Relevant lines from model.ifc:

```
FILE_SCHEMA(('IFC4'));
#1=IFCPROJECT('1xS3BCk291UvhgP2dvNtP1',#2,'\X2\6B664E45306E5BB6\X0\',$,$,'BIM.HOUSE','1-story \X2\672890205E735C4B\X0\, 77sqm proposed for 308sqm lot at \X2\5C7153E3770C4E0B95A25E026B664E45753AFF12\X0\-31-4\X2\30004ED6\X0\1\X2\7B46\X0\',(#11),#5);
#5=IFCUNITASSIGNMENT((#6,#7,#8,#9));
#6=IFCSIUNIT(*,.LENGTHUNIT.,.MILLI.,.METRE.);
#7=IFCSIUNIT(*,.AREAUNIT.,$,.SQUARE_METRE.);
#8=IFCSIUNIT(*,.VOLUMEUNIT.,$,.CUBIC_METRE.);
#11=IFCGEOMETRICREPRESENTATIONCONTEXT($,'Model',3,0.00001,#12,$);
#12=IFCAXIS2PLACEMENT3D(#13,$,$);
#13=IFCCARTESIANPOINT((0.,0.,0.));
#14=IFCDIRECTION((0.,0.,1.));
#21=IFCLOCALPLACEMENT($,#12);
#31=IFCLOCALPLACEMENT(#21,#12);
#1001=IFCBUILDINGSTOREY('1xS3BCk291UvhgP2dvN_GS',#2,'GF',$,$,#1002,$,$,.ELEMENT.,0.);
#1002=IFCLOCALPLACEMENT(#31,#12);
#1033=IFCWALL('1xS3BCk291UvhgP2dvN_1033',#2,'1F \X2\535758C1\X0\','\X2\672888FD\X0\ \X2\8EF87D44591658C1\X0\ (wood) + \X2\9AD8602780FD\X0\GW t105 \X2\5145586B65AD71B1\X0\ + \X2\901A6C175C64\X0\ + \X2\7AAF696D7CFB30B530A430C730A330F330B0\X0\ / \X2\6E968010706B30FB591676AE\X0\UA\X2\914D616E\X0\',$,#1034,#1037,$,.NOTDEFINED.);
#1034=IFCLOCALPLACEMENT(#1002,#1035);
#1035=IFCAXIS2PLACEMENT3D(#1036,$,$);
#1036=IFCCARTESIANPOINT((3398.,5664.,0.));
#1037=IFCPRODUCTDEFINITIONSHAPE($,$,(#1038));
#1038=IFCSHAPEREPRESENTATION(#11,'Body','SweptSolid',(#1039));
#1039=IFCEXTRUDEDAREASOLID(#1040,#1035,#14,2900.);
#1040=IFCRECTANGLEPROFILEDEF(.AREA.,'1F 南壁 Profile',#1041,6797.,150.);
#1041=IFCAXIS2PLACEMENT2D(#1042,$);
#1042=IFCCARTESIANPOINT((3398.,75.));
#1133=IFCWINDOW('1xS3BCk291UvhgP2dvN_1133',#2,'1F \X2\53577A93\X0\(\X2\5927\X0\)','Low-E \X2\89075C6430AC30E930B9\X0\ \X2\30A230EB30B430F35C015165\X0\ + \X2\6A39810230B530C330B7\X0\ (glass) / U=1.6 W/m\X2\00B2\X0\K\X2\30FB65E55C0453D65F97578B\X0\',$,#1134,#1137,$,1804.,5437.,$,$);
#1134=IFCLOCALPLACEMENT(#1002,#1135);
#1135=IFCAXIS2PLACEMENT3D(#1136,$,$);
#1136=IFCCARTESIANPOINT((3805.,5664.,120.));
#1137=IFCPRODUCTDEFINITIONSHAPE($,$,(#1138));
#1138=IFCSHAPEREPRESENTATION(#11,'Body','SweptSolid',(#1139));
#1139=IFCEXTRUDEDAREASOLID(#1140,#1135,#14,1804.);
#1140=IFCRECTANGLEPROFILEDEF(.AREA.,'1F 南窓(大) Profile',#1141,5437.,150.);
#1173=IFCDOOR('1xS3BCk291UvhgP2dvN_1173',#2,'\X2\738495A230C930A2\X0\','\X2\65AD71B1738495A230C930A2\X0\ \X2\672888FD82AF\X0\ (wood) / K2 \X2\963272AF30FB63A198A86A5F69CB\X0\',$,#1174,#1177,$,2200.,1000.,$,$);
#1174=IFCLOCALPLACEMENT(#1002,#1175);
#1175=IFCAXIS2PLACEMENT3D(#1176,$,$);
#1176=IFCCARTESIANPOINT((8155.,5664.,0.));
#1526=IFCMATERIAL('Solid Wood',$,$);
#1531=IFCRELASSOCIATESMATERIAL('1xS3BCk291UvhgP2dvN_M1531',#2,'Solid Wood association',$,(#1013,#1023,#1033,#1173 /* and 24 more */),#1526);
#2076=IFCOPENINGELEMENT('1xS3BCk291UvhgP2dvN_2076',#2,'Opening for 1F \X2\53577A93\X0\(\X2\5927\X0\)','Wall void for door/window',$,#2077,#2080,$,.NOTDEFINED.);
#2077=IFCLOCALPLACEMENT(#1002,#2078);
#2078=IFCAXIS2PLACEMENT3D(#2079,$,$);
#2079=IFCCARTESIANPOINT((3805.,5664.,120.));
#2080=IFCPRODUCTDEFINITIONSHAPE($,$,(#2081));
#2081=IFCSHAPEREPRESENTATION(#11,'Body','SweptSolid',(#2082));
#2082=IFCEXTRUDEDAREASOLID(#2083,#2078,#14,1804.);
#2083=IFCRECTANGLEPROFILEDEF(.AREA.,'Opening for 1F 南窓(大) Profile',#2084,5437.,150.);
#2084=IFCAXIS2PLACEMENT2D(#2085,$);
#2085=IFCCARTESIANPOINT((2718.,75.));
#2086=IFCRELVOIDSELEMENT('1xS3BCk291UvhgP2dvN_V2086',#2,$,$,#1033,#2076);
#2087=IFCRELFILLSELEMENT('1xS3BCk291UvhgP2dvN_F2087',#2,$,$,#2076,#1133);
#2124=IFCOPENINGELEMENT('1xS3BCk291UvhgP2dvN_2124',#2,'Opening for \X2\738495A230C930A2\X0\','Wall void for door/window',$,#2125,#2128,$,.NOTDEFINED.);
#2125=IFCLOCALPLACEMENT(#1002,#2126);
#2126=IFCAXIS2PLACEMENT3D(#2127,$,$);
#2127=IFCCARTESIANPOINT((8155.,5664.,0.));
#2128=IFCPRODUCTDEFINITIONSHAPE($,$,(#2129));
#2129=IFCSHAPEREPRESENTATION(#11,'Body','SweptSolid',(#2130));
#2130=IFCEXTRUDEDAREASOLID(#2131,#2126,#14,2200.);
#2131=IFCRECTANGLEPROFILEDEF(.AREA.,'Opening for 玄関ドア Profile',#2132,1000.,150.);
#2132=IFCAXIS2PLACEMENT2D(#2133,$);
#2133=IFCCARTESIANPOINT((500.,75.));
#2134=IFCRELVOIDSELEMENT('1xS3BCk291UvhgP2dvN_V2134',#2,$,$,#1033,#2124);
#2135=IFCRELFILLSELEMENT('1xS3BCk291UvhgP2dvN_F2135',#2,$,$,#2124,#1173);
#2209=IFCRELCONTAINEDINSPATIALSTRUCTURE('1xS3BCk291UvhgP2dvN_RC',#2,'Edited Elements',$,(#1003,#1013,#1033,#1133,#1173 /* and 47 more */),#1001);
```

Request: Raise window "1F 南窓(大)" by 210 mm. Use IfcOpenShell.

```python
import numpy as np
import ifcopenshell
import ifcopenshell.api.geometry
import ifcopenshell.util.placement
import ifcopenshell.util.unit

model = ifcopenshell.open("model.ifc")
unit_scale = ifcopenshell.util.unit.calculate_unit_scale(model)

window = model.by_guid("1xS3BCk291UvhgP2dvN_1133")
opening = window.FillsVoids[0].RelatingOpeningElement
dz = 0.21 / unit_scale

shift = np.array([0.0, 0.0, dz])
# The window is not placed relative to its opening, so move both.
for product in (opening, window):
    matrix = ifcopenshell.util.placement.get_local_placement(product.ObjectPlacement)
    matrix[:3, 3] += shift
    ifcopenshell.api.geometry.edit_object_placement(model, product=product, matrix=matrix, is_si=False)

print(f"moved by {dz * unit_scale:+.3f} m")

model.write("model_v2.ifc")
```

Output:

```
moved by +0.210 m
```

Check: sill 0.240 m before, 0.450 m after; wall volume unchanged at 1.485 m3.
